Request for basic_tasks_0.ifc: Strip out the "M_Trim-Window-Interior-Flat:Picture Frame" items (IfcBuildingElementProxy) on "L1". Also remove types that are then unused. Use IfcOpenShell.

First a look at what the model holds.

```python
import ifcopenshell
import ifcopenshell.util.element

model = ifcopenshell.open("basic_tasks_0.ifc")
print(model.schema)
storey = next(s for s in model.by_type("IfcBuildingStorey") if s.Name == "L1")
proxies = [e for e in ifcopenshell.util.element.get_decomposition(storey) if e.is_a("IfcBuildingElementProxy")]
seen = {}
for e in proxies:
    element_type = ifcopenshell.util.element.get_type(e)
    name = element_type.Name if element_type not in (None, e) else None
    seen[name] = seen.get(name, 0) + 1
for name, count in sorted(seen.items(), key=str):
    print(count, "x", name)
```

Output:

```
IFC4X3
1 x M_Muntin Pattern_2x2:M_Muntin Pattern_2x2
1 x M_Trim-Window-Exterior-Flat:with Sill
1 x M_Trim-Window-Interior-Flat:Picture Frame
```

```python
import ifcopenshell
import ifcopenshell.api.root
import ifcopenshell.util.element

model = ifcopenshell.open("basic_tasks_0.ifc")

storey = next(s for s in model.by_type("IfcBuildingStorey") if s.Name == "L1")
proxies = [e for e in ifcopenshell.util.element.get_decomposition(storey) if e.is_a("IfcBuildingElementProxy")]
targets = [e for e in proxies if (t := ifcopenshell.util.element.get_type(e)) not in (None, e) and t.Name == "M_Trim-Window-Interior-Flat:Picture Frame"]
types = {ifcopenshell.util.element.get_type(e) for e in targets} - {None, *targets}

for e in targets:
    ifcopenshell.api.root.remove_product(model, product=e)
print(len(targets), "removed")

unused = [t for t in types if not ifcopenshell.util.element.get_types(t)]
for t in unused:
    ifcopenshell.api.root.remove_product(model, product=t)
print(len(unused), "unused types removed")

model.write("basic_tasks_0_updated.ifc")
```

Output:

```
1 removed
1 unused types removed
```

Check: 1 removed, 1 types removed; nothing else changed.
